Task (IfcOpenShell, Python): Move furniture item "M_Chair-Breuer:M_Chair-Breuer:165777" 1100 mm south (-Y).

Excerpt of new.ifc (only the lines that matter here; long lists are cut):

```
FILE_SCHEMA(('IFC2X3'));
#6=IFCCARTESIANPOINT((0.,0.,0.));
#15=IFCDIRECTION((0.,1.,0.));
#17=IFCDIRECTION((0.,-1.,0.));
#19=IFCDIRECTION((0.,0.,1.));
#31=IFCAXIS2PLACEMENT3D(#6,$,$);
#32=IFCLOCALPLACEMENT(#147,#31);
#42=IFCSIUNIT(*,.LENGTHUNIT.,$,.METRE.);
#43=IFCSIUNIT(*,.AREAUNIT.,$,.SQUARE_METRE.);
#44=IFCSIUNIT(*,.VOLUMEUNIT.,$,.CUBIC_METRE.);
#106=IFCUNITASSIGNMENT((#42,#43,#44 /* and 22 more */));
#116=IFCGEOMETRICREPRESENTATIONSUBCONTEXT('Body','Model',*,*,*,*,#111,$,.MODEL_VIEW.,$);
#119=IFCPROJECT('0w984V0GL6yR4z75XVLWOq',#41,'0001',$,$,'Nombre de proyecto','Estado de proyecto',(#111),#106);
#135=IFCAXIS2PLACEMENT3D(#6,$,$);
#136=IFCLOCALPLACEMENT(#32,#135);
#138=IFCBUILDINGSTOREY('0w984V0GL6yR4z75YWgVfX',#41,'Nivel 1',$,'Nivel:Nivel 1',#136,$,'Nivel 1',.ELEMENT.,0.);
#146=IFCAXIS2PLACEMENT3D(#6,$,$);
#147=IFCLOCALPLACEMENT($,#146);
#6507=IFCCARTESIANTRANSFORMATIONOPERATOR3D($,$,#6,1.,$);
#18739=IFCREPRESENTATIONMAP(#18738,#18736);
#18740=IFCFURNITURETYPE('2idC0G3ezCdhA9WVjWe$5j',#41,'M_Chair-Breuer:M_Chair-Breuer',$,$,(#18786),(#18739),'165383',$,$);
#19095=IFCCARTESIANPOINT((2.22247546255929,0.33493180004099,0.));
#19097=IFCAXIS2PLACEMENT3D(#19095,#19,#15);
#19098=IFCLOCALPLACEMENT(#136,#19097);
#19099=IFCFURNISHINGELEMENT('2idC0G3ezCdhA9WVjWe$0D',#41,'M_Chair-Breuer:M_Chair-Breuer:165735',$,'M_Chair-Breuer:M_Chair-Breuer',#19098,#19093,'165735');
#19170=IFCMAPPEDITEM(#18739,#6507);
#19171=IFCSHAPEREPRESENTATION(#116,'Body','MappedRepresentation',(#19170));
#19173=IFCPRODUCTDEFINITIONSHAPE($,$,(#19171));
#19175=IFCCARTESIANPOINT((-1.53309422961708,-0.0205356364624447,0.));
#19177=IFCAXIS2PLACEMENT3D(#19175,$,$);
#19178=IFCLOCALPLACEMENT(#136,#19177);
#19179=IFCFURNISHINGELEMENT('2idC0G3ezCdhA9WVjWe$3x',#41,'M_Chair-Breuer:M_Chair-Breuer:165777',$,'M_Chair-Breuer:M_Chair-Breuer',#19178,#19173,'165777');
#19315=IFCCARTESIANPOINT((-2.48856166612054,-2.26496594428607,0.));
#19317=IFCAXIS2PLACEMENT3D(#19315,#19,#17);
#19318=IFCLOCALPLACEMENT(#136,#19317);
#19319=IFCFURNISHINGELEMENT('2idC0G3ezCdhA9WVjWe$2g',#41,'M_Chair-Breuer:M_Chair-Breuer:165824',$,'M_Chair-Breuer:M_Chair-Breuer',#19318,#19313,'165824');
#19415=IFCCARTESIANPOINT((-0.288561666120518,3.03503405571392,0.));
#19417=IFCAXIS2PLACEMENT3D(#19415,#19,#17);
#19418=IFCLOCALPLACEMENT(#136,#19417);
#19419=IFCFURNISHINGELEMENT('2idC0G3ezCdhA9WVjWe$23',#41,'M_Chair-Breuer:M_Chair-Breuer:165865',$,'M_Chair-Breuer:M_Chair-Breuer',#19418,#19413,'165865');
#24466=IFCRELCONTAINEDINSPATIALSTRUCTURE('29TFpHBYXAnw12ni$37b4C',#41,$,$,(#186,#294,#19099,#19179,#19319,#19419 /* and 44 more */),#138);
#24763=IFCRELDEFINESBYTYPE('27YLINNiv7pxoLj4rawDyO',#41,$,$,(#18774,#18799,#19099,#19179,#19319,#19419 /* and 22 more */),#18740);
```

```python
import ifcopenshell
import ifcopenshell.api.geometry
import ifcopenshell.util.placement
import ifcopenshell.util.unit

model = ifcopenshell.open("new.ifc")
unit_scale = ifcopenshell.util.unit.calculate_unit_scale(model)

item = model.by_id(19179)
matrix = ifcopenshell.util.placement.get_local_placement(item.ObjectPlacement)
matrix[1, 3] -= 1.1 / unit_scale
ifcopenshell.api.geometry.edit_object_placement(model, product=item, matrix=matrix, is_si=False)

print(ifcopenshell.util.placement.get_local_placement(item.ObjectPlacement).round(3) + 0.0)

model.write("new-out.ifc")
```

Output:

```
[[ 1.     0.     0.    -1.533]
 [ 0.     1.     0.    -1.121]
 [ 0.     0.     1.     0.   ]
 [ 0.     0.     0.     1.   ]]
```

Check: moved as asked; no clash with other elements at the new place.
